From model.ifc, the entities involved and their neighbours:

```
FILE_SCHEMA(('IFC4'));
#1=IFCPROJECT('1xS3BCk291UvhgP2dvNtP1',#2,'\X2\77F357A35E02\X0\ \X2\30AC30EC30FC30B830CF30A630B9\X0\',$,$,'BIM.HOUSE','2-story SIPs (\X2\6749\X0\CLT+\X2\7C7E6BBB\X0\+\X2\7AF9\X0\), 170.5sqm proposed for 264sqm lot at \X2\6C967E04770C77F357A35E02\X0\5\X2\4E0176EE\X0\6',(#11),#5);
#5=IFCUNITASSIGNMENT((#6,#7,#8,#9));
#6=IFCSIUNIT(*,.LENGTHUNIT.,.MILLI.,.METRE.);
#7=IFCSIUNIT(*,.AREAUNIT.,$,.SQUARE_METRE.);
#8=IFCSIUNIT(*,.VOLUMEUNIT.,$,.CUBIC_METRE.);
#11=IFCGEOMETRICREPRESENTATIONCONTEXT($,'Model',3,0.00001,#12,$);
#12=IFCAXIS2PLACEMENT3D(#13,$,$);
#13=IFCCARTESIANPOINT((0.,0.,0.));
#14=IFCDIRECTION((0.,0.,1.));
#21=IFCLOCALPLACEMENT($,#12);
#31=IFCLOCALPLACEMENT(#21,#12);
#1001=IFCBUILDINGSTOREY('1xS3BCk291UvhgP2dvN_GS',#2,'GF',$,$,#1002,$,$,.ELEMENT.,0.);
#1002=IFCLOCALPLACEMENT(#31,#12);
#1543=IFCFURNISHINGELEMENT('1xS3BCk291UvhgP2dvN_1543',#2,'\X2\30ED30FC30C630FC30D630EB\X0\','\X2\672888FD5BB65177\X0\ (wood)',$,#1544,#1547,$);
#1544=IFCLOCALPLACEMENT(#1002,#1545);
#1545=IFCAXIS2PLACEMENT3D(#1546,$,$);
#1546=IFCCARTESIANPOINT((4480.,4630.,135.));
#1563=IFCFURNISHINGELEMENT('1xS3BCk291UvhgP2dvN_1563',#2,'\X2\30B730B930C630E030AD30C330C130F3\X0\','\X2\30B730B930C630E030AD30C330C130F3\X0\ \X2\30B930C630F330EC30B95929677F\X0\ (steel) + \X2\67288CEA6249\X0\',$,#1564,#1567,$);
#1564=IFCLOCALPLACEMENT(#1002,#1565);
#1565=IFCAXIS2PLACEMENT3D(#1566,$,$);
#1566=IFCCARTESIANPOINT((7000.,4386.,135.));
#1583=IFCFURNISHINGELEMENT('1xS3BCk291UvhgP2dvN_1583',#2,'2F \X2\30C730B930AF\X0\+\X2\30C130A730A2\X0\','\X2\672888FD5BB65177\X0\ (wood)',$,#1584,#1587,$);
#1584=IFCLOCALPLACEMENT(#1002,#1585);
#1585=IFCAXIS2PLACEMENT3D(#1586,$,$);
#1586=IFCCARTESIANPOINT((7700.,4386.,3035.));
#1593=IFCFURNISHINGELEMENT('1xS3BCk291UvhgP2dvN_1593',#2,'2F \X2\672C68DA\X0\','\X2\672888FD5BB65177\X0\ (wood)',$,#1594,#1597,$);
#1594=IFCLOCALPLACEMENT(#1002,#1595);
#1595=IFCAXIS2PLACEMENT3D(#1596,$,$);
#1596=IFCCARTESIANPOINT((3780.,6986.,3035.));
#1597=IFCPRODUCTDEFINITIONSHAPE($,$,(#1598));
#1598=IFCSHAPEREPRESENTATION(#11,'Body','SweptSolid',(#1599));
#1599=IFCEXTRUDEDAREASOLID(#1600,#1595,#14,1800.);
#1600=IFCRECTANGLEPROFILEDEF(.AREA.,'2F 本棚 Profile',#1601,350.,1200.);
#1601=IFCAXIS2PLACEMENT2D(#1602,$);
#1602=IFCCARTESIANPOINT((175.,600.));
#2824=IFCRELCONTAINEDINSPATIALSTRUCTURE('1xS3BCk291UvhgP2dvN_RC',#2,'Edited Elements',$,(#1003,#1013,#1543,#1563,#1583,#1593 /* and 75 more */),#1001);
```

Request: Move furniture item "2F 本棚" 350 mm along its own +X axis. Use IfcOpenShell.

```python
import ifcopenshell
import ifcopenshell.api.geometry
import ifcopenshell.util.placement

model = ifcopenshell.open("model.ifc")

item = model.by_guid("1xS3BCk291UvhgP2dvN_1593")
matrix = ifcopenshell.util.placement.get_local_placement(item.ObjectPlacement)
matrix[:3, 3] += matrix[:3, 0] * 350.0
ifcopenshell.api.geometry.edit_object_placement(model, product=item, matrix=matrix, is_si=False)

print(ifcopenshell.util.placement.get_local_placement(item.ObjectPlacement).round(3) + 0.0)

model.write("model_edited.ifc")
```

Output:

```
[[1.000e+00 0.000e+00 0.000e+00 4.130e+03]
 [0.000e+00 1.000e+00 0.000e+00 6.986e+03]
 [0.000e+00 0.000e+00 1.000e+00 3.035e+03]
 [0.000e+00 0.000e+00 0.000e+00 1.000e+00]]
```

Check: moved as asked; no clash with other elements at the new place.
